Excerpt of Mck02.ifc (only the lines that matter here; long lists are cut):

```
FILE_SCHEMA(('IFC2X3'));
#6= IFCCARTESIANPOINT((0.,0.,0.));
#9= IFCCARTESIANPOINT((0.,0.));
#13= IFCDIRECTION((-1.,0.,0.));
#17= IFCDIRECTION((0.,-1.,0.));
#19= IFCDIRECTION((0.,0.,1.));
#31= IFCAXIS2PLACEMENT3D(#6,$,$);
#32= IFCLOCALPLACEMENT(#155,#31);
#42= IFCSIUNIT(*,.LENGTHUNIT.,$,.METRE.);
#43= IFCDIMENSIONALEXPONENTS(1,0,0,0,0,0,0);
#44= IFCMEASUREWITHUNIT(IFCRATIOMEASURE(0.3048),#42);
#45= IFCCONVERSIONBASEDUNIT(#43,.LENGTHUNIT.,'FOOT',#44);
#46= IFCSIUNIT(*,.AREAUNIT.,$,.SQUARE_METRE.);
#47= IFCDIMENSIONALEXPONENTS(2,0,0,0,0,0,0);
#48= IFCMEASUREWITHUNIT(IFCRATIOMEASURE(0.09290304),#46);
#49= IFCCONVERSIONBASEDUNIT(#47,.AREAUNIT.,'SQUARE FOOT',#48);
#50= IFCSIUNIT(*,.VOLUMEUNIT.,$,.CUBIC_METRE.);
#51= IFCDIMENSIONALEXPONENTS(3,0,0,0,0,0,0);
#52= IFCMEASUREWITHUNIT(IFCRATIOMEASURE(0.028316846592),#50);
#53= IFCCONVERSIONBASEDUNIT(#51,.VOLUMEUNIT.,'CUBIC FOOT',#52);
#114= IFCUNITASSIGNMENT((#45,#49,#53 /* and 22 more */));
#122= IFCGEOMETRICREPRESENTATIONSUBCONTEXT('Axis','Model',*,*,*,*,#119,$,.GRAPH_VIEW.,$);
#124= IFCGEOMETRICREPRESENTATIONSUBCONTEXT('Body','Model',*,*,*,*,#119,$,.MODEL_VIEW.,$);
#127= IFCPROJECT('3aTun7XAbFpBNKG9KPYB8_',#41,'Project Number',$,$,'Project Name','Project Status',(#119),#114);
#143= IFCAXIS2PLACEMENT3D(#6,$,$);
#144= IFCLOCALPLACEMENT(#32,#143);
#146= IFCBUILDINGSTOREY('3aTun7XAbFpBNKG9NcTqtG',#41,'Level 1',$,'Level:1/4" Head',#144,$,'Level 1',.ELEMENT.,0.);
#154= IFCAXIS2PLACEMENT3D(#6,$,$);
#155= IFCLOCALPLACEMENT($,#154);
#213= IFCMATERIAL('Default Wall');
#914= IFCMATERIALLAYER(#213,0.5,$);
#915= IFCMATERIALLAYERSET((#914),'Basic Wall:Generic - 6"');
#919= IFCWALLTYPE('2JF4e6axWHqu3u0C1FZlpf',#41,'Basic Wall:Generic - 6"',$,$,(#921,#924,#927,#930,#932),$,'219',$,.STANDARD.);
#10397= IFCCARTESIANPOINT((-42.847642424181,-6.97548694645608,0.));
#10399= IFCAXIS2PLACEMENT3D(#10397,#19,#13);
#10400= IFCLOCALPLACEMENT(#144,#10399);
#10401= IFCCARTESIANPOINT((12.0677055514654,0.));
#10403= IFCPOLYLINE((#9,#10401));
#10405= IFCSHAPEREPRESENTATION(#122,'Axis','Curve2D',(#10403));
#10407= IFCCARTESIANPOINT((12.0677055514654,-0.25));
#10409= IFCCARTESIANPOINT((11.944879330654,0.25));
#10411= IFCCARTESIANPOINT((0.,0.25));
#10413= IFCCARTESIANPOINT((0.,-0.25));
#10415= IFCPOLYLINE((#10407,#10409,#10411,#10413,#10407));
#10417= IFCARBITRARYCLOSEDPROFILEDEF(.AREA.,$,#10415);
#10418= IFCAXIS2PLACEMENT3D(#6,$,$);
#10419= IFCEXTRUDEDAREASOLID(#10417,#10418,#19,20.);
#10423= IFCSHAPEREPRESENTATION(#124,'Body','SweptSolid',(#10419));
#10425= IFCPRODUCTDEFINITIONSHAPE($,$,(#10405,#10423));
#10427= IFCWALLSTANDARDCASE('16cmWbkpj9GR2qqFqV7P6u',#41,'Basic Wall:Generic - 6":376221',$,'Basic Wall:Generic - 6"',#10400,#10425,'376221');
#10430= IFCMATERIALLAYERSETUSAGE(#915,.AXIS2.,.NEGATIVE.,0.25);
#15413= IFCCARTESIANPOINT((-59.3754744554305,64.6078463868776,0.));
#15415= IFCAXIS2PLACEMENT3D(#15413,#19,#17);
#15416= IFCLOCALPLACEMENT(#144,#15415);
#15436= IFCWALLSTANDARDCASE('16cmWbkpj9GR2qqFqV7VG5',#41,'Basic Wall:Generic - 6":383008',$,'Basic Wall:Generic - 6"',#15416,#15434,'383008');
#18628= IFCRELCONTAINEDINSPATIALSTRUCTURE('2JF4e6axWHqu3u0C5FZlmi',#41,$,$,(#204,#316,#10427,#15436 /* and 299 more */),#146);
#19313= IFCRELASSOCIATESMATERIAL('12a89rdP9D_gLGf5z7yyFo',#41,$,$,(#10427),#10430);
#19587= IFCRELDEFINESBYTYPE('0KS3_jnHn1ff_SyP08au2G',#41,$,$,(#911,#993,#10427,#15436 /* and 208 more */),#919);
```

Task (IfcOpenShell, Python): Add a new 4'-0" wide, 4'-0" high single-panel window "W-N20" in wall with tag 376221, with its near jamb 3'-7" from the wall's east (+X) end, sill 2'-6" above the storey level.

```python
import numpy as np
import ifcopenshell
import ifcopenshell.api.feature
import ifcopenshell.api.geometry
import ifcopenshell.api.root
import ifcopenshell.api.spatial
import ifcopenshell.api.type
import ifcopenshell.geom
import ifcopenshell.util.element
import ifcopenshell.util.placement
import ifcopenshell.util.representation
import ifcopenshell.util.shape
import ifcopenshell.util.unit

model = ifcopenshell.open("Mck02.ifc")
unit_scale = ifcopenshell.util.unit.calculate_unit_scale(model)
settings = ifcopenshell.geom.settings()


def volume(element):
    """Net volume in cubic metres, openings subtracted."""
    shape = ifcopenshell.geom.create_shape(settings, element)
    return ifcopenshell.util.shape.get_volume(shape.geometry)


wall = model.by_id(10427)
storey = ifcopenshell.util.element.get_container(wall, ifc_class="IfcBuildingStorey")
context = ifcopenshell.util.representation.get_context(model, "Model", "Body", "MODEL_VIEW")
before = volume(wall)

width, height, from_end, sill = 1.2192, 1.2192, 1.0922, 0.762  # metres

# The wall runs along its own X axis, and the end named is its -X end.
wall_shape = ifcopenshell.geom.create_shape(settings, wall)
x, y, z = ifcopenshell.util.shape.get_vertices(wall_shape.geometry).T
start = x.min() + from_end
face, thickness = float(y.min()), float(y.max() - y.min())
wall_matrix = ifcopenshell.util.placement.get_local_placement(wall.ObjectPlacement)
level = ifcopenshell.util.placement.get_local_placement(storey.ObjectPlacement)[2, 3]


def in_wall(x, y):
    """Placement at x, y metres in the wall's axes, at sill height."""
    matrix = wall_matrix.copy()
    matrix[:, 3] = wall_matrix @ np.array([x / unit_scale, y / unit_scale, 0.0, 1.0])
    matrix[2, 3] = level + sill / unit_scale
    return matrix


# Opening: a box that overshoots both wall faces by 50 mm.
opening = ifcopenshell.api.root.create_entity(model, ifc_class="IfcOpeningElement")
box = ifcopenshell.api.geometry.add_wall_representation(
    model, context=context, length=width, height=height, thickness=thickness + 0.1
)
ifcopenshell.api.geometry.assign_representation(model, product=opening, representation=box)
ifcopenshell.api.geometry.edit_object_placement(model, product=opening, matrix=in_wall(start, face - 0.05), is_si=False)
ifcopenshell.api.feature.add_feature(model, feature=opening, element=wall)

window = ifcopenshell.api.root.create_entity(model, ifc_class="IfcWindow", name="W-N20")
window.OverallWidth, window.OverallHeight = width / unit_scale, height / unit_scale
body = ifcopenshell.api.geometry.add_window_representation(
    model,
    context=context,
    overall_width=window.OverallWidth,
    overall_height=window.OverallHeight,
    partition_type="SINGLE_PANEL",
)
ifcopenshell.api.geometry.assign_representation(model, product=window, representation=body)
ifcopenshell.api.spatial.assign_container(model, products=[window], relating_structure=storey)
fills = ifcopenshell.api.feature.add_filling(model, opening=opening, element=window)
fills.OwnerHistory = window.OwnerHistory  # required in IFC2X3

# IFC2X3 keeps the operation on the window style.
style = ifcopenshell.api.root.create_entity(model, ifc_class="IfcWindowStyle", name="W-N20")
style.OperationType, style.ConstructionType = "SINGLE_PANEL", "NOTDEFINED"
style.ParameterTakesPrecedence = style.Sizeable = False
ifcopenshell.api.type.assign_type(model, related_objects=[window], relating_type=style)

# Centre the window in the wall's thickness.
ifcopenshell.api.geometry.edit_object_placement(model, product=window, matrix=in_wall(start, face), is_si=False)
window_shape = ifcopenshell.geom.create_shape(settings, window)
depth = ifcopenshell.util.shape.get_vertices(window_shape.geometry)[:, 1]
offset = face + thickness / 2 - (depth.min() + depth.max()) / 2
ifcopenshell.api.geometry.edit_object_placement(model, product=window, matrix=in_wall(start, offset), is_si=False)

after = volume(wall)

print(f"wall volume {before:.3f} -> {after:.3f} m3")

model.write("Mck02-out.ifc")
```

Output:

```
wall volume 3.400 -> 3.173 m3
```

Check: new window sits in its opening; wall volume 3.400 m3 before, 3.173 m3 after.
